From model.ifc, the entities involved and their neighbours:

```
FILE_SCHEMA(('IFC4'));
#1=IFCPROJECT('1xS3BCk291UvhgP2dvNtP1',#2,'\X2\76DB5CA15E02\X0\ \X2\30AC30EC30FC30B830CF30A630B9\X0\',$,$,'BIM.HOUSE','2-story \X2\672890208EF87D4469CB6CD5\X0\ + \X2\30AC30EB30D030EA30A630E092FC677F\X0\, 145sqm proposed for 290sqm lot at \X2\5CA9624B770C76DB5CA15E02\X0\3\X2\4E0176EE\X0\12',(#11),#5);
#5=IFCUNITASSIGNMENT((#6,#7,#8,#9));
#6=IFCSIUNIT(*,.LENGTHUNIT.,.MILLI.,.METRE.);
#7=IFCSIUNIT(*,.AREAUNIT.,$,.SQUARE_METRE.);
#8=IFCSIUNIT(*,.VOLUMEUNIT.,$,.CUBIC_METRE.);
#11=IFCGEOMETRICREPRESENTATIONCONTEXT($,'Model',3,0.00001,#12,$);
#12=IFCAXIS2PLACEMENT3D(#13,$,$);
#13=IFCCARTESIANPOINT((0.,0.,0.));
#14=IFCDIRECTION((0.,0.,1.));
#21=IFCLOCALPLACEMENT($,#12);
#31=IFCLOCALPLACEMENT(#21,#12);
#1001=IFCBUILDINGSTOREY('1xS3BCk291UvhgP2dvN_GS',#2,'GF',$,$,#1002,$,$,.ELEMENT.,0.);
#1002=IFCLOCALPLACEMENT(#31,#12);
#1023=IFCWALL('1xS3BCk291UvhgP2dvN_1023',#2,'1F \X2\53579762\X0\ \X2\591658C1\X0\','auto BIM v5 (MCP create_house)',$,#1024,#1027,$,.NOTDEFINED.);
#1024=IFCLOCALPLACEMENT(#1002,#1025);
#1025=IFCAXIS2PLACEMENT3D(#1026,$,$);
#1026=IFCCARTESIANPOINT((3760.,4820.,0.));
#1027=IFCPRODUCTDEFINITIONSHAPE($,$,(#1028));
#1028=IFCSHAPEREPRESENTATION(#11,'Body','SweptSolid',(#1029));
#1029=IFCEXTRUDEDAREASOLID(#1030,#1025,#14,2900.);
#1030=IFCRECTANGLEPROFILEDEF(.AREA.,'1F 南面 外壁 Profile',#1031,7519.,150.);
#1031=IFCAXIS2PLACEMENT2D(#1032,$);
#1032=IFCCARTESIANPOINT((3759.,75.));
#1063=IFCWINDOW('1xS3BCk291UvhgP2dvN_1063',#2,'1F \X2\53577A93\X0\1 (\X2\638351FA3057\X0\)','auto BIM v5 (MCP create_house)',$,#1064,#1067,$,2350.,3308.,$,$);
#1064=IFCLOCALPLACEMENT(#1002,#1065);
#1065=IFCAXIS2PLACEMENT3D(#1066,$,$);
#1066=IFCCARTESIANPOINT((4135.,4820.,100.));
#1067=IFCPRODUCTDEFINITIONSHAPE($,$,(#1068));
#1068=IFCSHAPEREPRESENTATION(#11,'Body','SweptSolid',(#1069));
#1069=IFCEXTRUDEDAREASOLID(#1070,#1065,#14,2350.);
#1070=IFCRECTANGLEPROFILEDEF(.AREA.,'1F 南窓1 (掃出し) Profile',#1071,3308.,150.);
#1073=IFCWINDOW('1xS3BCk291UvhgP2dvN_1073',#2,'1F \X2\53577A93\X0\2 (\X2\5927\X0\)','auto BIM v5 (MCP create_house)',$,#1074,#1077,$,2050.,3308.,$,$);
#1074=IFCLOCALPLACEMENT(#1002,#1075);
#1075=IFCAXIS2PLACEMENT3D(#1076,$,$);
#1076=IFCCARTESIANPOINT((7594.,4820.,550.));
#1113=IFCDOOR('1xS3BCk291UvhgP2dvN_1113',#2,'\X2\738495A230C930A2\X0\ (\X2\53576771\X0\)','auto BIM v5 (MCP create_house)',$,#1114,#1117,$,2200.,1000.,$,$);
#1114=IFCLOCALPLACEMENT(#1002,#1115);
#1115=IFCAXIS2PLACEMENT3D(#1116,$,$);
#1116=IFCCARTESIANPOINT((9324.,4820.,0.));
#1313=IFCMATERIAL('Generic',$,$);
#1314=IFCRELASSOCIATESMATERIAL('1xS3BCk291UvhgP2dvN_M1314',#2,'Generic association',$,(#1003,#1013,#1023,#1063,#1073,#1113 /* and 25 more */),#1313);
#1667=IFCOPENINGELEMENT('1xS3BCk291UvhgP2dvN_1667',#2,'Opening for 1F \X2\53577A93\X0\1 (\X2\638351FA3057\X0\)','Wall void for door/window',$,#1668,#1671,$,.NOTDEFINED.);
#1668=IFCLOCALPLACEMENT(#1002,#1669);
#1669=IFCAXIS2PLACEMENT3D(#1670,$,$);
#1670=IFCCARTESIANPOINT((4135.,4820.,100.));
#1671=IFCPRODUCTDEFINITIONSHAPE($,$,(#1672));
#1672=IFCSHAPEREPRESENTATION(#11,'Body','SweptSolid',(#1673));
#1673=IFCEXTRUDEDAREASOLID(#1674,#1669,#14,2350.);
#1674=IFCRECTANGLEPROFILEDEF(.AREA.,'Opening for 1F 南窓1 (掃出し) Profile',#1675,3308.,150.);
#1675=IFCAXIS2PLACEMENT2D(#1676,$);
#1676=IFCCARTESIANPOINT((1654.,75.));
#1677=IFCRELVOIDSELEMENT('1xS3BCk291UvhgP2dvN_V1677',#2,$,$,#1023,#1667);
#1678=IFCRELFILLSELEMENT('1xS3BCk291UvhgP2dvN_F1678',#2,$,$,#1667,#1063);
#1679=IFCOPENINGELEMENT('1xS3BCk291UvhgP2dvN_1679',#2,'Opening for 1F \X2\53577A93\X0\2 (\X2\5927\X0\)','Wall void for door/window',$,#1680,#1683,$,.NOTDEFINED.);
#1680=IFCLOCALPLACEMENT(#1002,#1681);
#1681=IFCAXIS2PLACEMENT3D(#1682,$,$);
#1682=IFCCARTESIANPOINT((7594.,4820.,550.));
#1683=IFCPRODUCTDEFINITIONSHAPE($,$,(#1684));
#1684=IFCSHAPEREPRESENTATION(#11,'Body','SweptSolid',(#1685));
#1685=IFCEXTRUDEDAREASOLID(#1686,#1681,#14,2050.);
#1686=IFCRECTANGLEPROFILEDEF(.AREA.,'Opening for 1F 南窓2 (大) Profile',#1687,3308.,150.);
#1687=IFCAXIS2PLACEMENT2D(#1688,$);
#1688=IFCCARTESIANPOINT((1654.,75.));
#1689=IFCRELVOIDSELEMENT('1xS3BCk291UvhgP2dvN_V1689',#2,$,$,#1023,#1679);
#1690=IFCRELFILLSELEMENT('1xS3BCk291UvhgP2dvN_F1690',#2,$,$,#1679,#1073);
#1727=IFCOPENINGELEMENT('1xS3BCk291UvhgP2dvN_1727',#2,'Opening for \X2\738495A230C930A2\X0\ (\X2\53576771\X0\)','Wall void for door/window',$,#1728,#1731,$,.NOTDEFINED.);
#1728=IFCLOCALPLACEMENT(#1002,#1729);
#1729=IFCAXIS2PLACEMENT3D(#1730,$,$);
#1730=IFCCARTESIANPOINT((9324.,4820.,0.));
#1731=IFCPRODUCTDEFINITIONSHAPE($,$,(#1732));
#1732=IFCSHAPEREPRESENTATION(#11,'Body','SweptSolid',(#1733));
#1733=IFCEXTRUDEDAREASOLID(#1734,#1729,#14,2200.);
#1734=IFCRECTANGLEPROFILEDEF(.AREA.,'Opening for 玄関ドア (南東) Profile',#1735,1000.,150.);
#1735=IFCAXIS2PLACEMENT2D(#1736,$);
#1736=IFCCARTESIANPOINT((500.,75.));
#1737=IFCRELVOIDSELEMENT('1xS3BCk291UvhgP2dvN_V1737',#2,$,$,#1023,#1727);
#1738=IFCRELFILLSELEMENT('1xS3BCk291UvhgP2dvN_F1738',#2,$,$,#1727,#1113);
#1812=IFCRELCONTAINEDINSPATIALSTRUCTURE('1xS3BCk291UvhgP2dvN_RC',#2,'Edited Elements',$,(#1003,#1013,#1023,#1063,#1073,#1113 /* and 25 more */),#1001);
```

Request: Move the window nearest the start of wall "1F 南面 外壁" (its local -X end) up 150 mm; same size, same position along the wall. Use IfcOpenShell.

```python
import numpy as np
import ifcopenshell
import ifcopenshell.api.geometry
import ifcopenshell.util.placement
import ifcopenshell.util.unit

model = ifcopenshell.open("model.ifc")
unit_scale = ifcopenshell.util.unit.calculate_unit_scale(model)

window = model.by_id(1063)
opening = window.FillsVoids[0].RelatingOpeningElement
dz = 0.15 / unit_scale

shift = np.array([0.0, 0.0, dz])
# The window is not placed relative to its opening, so move both.
for product in (opening, window):
    matrix = ifcopenshell.util.placement.get_local_placement(product.ObjectPlacement)
    matrix[:3, 3] += shift
    ifcopenshell.api.geometry.edit_object_placement(model, product=product, matrix=matrix, is_si=False)

print(f"moved by {dz * unit_scale:+.3f} m")

model.write("model_v2.ifc")
```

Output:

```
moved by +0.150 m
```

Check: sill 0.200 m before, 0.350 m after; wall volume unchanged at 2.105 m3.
